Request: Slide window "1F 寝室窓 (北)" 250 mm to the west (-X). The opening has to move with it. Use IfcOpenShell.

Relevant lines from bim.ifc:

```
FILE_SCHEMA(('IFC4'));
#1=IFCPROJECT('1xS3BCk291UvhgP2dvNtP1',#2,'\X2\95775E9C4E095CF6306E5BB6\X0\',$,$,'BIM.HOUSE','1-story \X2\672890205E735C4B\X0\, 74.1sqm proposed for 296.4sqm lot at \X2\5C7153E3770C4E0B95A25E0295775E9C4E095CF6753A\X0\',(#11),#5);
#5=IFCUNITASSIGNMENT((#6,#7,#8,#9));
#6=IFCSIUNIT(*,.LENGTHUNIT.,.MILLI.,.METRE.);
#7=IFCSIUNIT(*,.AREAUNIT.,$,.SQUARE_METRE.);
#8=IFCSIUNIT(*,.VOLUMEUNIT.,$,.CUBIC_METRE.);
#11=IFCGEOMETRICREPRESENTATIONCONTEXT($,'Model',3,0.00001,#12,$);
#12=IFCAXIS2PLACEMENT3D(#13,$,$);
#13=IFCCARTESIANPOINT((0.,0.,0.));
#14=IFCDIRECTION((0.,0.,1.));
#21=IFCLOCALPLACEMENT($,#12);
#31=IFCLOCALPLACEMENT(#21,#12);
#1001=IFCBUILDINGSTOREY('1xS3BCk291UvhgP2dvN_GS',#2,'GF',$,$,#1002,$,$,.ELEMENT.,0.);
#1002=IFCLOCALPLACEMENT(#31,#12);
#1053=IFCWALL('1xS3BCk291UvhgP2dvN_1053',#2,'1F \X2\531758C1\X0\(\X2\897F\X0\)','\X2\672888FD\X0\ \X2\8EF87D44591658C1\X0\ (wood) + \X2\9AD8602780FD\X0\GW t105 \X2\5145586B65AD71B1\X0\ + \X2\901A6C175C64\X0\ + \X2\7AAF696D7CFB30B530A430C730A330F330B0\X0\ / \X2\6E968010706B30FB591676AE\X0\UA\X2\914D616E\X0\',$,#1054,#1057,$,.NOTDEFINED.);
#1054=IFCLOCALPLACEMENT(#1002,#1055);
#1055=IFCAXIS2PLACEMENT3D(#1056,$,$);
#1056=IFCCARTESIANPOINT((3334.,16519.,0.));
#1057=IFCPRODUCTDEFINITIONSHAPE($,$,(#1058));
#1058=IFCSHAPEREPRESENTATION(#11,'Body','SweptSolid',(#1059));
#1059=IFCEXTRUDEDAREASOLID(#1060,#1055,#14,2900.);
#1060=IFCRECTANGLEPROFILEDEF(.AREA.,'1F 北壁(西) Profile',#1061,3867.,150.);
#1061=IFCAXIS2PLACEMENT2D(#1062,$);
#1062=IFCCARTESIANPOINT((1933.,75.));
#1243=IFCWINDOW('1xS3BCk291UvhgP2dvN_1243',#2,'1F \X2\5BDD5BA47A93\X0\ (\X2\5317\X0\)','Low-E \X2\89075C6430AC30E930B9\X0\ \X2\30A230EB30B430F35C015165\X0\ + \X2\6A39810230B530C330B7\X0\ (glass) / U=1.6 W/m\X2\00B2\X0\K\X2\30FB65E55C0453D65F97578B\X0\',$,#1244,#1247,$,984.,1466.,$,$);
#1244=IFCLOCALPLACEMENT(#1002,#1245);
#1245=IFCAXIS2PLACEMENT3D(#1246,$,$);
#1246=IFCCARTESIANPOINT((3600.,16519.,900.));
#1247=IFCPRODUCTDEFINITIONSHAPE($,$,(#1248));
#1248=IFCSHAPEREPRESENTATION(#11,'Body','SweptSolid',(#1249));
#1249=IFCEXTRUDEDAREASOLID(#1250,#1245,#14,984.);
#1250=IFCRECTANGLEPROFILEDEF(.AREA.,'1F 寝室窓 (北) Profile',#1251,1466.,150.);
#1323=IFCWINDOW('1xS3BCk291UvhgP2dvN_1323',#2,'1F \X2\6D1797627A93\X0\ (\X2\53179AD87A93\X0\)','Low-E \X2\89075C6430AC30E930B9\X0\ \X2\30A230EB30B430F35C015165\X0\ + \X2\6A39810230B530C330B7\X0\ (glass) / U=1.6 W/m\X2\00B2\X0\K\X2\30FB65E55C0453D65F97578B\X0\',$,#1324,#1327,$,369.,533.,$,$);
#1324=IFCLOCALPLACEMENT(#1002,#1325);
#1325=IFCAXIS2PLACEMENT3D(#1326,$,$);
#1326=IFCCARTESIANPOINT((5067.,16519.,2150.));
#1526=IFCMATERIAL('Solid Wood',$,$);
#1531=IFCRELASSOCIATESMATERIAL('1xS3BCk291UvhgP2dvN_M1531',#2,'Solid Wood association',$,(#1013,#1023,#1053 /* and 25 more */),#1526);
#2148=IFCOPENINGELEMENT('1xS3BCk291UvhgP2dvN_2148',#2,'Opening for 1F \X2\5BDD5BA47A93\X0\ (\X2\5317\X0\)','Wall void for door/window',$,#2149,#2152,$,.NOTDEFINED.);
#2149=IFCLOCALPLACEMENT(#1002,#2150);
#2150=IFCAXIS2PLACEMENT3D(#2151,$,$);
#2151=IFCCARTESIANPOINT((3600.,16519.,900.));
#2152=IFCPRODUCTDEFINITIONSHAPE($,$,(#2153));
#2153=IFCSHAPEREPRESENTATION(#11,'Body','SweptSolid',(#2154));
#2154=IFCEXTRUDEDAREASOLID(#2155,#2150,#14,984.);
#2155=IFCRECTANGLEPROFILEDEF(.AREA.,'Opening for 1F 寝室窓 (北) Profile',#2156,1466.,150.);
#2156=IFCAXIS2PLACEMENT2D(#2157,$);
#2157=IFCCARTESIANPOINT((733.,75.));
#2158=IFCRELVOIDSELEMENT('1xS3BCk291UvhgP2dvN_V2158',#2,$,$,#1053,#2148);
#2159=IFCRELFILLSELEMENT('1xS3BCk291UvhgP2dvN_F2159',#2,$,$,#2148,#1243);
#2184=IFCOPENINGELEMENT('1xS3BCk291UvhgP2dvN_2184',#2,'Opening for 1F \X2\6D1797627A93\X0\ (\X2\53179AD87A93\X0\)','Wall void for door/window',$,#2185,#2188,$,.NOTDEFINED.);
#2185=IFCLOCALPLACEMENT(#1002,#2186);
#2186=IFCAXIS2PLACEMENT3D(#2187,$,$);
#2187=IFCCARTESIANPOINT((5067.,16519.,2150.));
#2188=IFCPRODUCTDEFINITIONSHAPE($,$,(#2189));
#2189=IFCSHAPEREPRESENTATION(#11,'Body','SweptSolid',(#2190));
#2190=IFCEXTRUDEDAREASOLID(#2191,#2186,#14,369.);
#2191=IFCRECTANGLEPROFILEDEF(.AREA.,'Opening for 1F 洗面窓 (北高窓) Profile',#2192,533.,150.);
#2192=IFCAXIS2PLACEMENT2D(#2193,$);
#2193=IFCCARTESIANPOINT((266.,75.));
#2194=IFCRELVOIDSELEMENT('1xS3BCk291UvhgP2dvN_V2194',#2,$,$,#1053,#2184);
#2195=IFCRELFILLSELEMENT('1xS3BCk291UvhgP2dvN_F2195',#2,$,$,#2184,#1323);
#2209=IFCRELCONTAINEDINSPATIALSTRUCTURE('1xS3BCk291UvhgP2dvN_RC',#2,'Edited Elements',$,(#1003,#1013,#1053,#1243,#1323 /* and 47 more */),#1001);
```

```python
import ifcopenshell
import ifcopenshell.api.geometry
import ifcopenshell.util.placement
import ifcopenshell.util.unit

model = ifcopenshell.open("bim.ifc")
unit_scale = ifcopenshell.util.unit.calculate_unit_scale(model)

window = model.by_id(1243)
opening = window.FillsVoids[0].RelatingOpeningElement
wall = opening.VoidsElements[0].RelatingBuildingElement

wall_matrix = ifcopenshell.util.placement.get_local_placement(wall.ObjectPlacement)
shift = wall_matrix[:3, 0] * -0.25 / unit_scale
before = ifcopenshell.util.placement.get_local_placement(window.ObjectPlacement)[:3, 3].copy()

# The window is not placed relative to its opening, so move both.
for product in (opening, window):
    matrix = ifcopenshell.util.placement.get_local_placement(product.ObjectPlacement)
    matrix[:3, 3] += shift
    ifcopenshell.api.geometry.edit_object_placement(model, product=product, matrix=matrix, is_si=False)

after = ifcopenshell.util.placement.get_local_placement(window.ObjectPlacement)[:3, 3]
print("window moved by", (after - before).round(3) + 0.0)

model.write("bim_v2.ifc")
```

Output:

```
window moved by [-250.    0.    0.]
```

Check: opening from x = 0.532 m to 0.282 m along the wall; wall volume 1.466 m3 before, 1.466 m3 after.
